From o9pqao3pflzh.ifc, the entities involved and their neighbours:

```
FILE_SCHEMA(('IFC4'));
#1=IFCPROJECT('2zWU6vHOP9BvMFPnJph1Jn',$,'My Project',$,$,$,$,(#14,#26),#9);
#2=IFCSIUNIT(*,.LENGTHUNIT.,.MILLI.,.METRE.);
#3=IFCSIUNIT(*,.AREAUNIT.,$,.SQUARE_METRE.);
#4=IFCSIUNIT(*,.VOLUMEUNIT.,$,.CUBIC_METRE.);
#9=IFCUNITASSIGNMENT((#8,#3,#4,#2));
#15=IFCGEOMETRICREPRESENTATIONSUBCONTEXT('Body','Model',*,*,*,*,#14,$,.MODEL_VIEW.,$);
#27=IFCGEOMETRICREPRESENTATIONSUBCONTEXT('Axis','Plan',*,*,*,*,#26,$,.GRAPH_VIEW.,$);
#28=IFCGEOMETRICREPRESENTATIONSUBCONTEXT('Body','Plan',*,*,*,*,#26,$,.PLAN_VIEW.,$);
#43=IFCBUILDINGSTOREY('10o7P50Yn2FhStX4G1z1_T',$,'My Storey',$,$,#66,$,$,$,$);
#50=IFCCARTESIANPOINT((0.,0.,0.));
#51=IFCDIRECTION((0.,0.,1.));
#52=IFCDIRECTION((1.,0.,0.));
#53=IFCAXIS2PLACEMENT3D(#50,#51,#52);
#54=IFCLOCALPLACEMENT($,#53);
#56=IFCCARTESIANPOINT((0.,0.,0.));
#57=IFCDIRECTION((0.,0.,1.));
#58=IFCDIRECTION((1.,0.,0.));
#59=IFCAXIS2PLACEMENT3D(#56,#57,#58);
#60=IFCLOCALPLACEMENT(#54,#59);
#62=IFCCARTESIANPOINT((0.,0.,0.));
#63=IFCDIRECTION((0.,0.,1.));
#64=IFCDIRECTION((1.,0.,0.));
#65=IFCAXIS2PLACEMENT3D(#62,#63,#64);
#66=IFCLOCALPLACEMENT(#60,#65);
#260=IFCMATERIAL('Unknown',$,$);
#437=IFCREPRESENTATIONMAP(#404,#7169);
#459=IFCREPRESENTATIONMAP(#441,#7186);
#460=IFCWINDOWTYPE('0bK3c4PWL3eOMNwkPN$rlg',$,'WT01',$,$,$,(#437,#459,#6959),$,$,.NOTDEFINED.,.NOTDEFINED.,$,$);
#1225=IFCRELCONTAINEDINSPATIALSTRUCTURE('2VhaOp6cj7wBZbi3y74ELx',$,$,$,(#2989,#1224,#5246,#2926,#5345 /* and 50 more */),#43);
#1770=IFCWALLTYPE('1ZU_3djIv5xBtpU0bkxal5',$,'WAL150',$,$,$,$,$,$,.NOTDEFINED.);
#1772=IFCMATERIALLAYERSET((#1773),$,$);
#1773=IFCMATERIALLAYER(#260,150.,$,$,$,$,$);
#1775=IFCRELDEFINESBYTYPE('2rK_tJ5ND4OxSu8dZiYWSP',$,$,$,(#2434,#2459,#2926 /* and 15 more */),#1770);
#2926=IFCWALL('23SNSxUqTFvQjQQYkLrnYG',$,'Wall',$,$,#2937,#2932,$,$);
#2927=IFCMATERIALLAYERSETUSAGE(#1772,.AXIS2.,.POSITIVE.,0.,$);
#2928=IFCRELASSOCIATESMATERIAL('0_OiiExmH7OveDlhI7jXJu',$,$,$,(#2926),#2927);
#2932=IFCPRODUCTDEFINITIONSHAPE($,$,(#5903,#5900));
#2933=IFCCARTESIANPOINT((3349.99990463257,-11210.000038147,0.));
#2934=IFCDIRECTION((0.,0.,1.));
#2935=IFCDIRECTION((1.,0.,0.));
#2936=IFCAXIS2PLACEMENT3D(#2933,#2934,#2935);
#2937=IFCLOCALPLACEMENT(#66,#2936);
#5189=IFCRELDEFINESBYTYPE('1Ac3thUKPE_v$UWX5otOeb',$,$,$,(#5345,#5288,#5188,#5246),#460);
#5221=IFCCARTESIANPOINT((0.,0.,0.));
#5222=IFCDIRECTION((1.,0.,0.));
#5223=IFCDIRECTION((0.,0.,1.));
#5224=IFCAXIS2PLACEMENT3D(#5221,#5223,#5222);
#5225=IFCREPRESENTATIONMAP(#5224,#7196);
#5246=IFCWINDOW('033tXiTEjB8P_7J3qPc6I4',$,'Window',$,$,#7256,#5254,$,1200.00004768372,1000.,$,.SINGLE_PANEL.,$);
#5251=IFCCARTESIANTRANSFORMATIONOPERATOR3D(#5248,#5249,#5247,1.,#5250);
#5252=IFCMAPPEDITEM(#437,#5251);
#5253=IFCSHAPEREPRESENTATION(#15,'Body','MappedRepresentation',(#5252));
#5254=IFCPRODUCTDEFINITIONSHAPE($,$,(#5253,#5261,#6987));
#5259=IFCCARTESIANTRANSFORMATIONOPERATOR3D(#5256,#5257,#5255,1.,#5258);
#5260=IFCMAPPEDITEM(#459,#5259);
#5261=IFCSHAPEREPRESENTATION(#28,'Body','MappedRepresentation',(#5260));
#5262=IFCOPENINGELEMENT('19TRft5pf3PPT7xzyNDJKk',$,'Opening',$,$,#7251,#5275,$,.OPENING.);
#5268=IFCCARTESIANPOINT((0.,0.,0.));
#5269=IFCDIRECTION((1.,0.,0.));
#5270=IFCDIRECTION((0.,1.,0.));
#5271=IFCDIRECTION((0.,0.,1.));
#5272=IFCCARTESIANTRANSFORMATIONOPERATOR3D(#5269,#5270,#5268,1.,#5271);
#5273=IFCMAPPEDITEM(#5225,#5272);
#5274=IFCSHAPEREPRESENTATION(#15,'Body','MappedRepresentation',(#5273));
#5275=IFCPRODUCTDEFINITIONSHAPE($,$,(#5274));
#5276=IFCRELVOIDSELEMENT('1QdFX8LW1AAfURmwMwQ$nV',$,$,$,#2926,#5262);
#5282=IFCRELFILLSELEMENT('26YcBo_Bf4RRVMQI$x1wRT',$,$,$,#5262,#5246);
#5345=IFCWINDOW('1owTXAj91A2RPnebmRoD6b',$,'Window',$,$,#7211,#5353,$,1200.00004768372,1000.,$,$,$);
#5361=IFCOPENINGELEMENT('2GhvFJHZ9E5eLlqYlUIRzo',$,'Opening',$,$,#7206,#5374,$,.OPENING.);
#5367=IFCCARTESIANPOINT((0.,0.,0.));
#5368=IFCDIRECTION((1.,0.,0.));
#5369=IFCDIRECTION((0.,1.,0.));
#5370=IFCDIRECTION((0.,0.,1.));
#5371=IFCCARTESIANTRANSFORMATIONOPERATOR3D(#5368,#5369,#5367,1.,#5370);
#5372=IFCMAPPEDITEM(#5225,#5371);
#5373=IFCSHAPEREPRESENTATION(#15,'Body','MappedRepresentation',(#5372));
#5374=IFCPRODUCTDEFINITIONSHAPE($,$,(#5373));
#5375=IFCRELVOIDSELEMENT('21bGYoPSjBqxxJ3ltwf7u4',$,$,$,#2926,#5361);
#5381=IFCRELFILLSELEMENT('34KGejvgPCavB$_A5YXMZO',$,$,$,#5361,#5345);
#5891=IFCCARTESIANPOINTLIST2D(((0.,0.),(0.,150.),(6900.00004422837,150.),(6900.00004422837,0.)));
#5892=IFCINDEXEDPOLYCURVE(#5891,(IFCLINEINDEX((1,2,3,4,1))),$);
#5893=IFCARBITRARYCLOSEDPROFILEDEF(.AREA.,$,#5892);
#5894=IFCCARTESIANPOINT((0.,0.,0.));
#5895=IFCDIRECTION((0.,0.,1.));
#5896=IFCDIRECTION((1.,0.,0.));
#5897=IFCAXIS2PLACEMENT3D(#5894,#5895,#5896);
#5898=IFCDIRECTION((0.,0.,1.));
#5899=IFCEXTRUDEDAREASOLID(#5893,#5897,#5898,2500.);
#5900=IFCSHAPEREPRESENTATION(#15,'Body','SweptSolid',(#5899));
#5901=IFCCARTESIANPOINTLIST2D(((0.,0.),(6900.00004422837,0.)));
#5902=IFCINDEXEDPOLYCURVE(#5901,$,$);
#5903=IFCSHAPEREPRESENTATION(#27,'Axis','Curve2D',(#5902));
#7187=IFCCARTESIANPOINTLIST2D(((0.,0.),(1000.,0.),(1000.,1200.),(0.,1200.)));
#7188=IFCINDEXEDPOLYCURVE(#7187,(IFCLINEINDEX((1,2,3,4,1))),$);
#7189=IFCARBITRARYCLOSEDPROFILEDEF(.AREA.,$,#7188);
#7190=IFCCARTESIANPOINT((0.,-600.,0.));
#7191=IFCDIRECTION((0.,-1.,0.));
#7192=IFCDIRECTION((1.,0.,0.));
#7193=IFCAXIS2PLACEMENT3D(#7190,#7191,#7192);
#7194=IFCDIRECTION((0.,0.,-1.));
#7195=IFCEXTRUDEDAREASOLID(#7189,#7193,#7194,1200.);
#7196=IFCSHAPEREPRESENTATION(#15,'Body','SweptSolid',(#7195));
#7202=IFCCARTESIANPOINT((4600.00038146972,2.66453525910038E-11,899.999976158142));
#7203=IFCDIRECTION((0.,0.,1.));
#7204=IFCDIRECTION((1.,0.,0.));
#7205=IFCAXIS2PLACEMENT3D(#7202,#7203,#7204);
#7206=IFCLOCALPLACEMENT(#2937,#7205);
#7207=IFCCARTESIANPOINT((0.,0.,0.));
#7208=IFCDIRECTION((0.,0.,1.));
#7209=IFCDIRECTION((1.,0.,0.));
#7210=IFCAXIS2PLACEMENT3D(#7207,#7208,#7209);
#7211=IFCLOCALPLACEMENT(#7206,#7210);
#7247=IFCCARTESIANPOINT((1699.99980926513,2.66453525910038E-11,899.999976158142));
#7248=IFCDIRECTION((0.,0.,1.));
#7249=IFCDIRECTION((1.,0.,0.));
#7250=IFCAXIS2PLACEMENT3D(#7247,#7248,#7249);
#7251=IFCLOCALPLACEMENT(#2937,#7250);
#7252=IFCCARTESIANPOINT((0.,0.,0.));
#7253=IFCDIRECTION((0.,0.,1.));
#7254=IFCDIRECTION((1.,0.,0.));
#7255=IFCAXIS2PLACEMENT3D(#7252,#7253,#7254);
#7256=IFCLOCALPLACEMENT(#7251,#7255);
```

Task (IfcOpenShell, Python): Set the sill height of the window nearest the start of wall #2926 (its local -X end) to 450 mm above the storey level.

```python
import numpy as np
import ifcopenshell
import ifcopenshell.api.geometry
import ifcopenshell.geom
import ifcopenshell.util.element
import ifcopenshell.util.placement
import ifcopenshell.util.shape
import ifcopenshell.util.unit

model = ifcopenshell.open("o9pqao3pflzh.ifc")
unit_scale = ifcopenshell.util.unit.calculate_unit_scale(model)

window = model.by_guid("033tXiTEjB8P_7J3qPc6I4")
opening = window.FillsVoids[0].RelatingOpeningElement
storey = ifcopenshell.util.element.get_container(window, ifc_class="IfcBuildingStorey")
level = ifcopenshell.util.placement.get_local_placement(storey.ObjectPlacement)[2, 3]

# The opening's origin need not be at the sill, so measure its lowest point.
shape = ifcopenshell.geom.create_shape(ifcopenshell.geom.settings(), opening)
bottom = ifcopenshell.util.shape.get_shape_bottom_elevation(shape, shape.geometry) / unit_scale
dz = level + 450.0 - bottom

shift = np.array([0.0, 0.0, dz])
# The window is placed relative to its opening, so it follows when the opening moves.
matrix = ifcopenshell.util.placement.get_local_placement(opening.ObjectPlacement)
matrix[:3, 3] += shift
ifcopenshell.api.geometry.edit_object_placement(
    model, product=opening, matrix=matrix, is_si=False, should_transform_children=True
)

print(f"moved by {dz * unit_scale:+.3f} m")

model.write("o9pqao3pflzh-out.ifc")
```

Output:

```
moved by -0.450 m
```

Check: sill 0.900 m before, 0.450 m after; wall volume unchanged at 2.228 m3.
